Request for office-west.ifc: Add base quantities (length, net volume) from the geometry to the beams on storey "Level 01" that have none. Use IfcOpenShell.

First a look at what the model holds.

```python
import ifcopenshell
import ifcopenshell.util.element
import ifcopenshell.util.unit

model = ifcopenshell.open("office-west.ifc")
print(model.schema)
for unit_type in ("LENGTHUNIT", "AREAUNIT", "VOLUMEUNIT"):
    print(unit_type, ifcopenshell.util.unit.calculate_unit_scale(model, unit_type))
storey = next(s for s in model.by_type("IfcBuildingStorey") if s.Name == "Level 01")
beams = [e for e in ifcopenshell.util.element.get_decomposition(storey) if e.is_a("IfcBeam")]
for e in sorted(beams, key=lambda e: e.id()):
    print(e.id(), e.is_a(), e.Name, list(ifcopenshell.util.element.get_psets(e, qtos_only=True)), sep=" | ")
```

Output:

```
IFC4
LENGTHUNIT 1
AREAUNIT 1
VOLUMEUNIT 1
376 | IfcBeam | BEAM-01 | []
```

```python
import ifcopenshell
import ifcopenshell.api.pset
import ifcopenshell.geom
import ifcopenshell.util.element
import ifcopenshell.util.shape
import ifcopenshell.util.unit

model = ifcopenshell.open("office-west.ifc")
unit_scale = ifcopenshell.util.unit.calculate_unit_scale(model)
volume_scale = ifcopenshell.util.unit.calculate_unit_scale(model, "VOLUMEUNIT")
settings = ifcopenshell.geom.settings()

storey = next(s for s in model.by_type("IfcBuildingStorey") if s.Name == "Level 01")
beams = [e for e in ifcopenshell.util.element.get_decomposition(storey) if e.is_a("IfcBeam")]

for e in sorted(beams, key=lambda e: e.id()):
    if ifcopenshell.util.element.get_psets(e, qtos_only=True, should_inherit=False):
        continue
    # Geometry comes back in metres, in the element's own axes.
    shape = ifcopenshell.geom.create_shape(settings, e)
    values = {
        "Length": ifcopenshell.util.shape.get_max_xyz(shape.geometry) / unit_scale,
        "NetVolume": ifcopenshell.util.shape.get_volume(shape.geometry) / volume_scale,
    }
    qto = ifcopenshell.api.pset.add_qto(model, product=e, name="Qto_BeamBaseQuantities")
    ifcopenshell.api.pset.edit_qto(model, qto=qto, properties=values)
    print(e.id(), {k: round(v, 3) for k, v in values.items()})

model.write("office-west_edited.ifc")
```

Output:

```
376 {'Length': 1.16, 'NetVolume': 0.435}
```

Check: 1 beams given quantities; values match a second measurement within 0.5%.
